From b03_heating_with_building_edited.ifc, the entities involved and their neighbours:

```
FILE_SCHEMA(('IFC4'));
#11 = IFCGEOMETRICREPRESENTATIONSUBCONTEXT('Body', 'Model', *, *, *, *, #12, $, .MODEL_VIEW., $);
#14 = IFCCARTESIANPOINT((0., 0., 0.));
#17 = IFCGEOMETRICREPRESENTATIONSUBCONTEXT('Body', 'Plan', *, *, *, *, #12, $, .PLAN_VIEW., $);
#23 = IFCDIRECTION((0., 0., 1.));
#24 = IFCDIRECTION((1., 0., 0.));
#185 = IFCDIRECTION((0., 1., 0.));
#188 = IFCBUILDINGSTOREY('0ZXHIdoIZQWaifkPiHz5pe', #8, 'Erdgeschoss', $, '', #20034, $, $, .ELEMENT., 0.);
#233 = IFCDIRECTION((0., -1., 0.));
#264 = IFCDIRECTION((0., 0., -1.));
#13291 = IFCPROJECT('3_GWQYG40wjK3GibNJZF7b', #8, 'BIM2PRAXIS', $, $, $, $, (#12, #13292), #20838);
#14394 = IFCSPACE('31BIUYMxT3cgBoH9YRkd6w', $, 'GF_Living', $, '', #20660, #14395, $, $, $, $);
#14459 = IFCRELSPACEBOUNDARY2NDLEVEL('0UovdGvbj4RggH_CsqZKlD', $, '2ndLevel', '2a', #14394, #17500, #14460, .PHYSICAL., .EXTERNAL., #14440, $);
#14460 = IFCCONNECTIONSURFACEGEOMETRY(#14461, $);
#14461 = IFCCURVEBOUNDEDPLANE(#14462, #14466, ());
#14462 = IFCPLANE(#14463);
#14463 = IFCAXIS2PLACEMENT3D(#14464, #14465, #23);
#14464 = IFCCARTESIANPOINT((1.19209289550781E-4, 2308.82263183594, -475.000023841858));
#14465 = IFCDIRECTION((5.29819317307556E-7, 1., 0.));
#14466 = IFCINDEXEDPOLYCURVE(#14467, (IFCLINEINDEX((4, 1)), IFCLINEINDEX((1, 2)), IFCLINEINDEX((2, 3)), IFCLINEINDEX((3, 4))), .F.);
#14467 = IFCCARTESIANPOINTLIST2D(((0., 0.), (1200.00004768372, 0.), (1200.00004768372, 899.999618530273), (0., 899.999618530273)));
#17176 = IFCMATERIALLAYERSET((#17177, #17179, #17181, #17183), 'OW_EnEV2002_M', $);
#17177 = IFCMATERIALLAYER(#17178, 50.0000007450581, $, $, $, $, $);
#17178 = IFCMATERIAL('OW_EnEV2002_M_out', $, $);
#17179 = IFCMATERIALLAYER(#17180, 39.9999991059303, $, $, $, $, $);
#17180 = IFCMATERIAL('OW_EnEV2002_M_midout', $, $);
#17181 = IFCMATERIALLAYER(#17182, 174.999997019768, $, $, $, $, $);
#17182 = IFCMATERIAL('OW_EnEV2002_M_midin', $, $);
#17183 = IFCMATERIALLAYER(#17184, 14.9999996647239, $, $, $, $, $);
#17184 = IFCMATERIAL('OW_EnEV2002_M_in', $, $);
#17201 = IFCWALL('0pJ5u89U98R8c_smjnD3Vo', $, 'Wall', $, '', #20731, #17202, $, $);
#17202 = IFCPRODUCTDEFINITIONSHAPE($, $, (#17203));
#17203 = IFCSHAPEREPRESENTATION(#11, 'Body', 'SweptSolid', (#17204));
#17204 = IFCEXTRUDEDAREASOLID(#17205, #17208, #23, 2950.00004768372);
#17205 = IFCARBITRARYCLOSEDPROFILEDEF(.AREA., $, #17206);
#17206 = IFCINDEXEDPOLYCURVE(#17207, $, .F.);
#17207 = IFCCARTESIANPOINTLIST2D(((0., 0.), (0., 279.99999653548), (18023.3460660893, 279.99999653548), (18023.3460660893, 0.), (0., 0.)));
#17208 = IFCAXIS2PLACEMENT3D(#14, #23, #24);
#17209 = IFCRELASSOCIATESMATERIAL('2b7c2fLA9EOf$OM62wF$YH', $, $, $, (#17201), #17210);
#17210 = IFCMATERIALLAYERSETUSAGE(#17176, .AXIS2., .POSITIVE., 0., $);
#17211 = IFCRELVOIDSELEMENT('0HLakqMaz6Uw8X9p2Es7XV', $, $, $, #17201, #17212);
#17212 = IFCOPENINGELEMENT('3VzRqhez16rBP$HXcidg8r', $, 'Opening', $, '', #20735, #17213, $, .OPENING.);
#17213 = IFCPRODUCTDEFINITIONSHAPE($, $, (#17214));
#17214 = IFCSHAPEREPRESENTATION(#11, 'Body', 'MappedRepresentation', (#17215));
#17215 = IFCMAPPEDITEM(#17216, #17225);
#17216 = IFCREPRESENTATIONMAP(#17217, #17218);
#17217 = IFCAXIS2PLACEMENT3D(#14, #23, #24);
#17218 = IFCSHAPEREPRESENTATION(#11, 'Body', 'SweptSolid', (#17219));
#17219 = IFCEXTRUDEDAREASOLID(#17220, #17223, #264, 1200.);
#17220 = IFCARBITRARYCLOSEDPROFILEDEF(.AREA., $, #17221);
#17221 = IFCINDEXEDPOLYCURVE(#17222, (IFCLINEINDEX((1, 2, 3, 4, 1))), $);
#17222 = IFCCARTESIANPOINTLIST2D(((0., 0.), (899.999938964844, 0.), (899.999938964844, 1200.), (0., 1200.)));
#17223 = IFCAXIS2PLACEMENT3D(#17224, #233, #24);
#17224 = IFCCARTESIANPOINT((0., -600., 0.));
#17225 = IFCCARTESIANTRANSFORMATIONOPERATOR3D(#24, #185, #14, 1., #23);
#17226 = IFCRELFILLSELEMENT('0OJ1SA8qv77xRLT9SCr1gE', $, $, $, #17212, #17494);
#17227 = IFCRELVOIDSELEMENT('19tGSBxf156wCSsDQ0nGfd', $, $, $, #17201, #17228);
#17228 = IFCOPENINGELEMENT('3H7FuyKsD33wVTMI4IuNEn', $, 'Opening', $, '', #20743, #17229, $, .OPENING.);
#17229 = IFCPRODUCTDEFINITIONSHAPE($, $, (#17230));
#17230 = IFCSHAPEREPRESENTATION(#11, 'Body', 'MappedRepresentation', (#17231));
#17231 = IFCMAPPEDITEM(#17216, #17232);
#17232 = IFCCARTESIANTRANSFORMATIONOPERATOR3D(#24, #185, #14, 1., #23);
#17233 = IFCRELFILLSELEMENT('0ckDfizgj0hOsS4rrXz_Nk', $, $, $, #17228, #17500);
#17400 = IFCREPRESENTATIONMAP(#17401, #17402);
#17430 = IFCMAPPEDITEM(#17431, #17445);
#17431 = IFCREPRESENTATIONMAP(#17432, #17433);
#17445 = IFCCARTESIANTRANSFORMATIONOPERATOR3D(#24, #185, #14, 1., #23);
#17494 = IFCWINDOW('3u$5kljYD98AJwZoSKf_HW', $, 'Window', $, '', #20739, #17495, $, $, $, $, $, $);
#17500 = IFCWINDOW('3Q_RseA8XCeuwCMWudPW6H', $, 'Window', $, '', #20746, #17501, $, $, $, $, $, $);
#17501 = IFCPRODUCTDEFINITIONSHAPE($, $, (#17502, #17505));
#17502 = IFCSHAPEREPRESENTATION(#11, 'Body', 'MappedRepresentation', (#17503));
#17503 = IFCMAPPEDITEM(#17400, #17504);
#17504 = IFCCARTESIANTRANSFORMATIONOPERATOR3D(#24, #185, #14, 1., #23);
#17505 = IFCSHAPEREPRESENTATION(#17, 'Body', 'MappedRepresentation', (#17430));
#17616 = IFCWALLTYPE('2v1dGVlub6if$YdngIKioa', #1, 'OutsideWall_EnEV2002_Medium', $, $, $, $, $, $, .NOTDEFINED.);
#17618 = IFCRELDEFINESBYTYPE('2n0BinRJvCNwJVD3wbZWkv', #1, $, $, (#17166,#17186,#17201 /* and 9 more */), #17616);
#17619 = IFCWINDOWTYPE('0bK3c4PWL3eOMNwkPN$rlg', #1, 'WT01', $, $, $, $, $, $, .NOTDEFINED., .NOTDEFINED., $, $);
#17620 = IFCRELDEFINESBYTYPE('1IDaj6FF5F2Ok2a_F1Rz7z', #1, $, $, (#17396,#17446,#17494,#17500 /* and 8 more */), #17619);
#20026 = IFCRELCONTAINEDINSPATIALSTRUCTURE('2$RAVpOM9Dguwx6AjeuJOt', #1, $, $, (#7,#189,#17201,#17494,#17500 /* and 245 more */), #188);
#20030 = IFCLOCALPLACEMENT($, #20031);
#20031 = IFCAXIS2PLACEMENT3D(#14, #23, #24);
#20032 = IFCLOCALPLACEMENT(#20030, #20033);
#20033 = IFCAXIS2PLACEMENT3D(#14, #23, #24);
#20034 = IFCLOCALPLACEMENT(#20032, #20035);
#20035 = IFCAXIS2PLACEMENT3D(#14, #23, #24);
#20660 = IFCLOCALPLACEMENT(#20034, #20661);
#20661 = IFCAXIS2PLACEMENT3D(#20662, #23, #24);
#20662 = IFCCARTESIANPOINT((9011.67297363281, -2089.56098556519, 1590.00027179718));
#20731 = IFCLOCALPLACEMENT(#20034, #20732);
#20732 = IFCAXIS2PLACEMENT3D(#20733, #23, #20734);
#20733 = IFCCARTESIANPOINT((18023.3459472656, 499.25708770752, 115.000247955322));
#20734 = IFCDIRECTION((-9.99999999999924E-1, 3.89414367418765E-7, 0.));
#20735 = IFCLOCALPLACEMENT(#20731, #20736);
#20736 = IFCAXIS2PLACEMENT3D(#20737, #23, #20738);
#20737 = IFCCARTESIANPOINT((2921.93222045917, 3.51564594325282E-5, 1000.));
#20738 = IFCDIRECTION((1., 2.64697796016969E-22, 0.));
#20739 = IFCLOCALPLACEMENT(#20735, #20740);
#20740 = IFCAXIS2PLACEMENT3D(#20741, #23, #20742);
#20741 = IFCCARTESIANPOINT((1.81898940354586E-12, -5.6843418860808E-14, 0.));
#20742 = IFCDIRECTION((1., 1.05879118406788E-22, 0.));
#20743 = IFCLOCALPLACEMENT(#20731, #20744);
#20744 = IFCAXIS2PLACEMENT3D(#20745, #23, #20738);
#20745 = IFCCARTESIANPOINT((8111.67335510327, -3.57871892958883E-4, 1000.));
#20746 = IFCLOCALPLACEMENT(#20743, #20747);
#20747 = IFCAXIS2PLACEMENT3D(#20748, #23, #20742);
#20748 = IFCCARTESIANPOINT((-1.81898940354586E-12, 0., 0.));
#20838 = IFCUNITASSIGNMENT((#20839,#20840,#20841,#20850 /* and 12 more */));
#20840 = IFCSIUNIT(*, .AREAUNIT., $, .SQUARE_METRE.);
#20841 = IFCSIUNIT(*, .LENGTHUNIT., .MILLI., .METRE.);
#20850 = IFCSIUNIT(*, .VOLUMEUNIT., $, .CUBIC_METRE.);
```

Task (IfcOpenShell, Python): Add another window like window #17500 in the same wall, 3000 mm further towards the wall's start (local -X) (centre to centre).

```python
import numpy as np
import ifcopenshell
import ifcopenshell.api.feature
import ifcopenshell.api.geometry
import ifcopenshell.api.root
import ifcopenshell.geom
import ifcopenshell.util.element
import ifcopenshell.util.placement
import ifcopenshell.util.shape

model = ifcopenshell.open("b03_heating_with_building_edited.ifc")
settings = ifcopenshell.geom.settings()


def volume(element):
    """Net volume in cubic metres, openings subtracted."""
    shape = ifcopenshell.geom.create_shape(settings, element)
    return ifcopenshell.util.shape.get_volume(shape.geometry)


def reuse_history(source, copy):
    """copy_class also copies each property set's owner history, people and application; keep the originals."""
    for rel in copy.IsDefinedBy:
        if rel.is_a("IfcRelDefinesByProperties") and (history := rel.RelatingPropertyDefinition.OwnerHistory):
            rel.RelatingPropertyDefinition.OwnerHistory = source.OwnerHistory
            ifcopenshell.util.element.remove_deep2(model, history)


window = model.by_guid("3Q_RseA8XCeuwCMWudPW6H")
opening = window.FillsVoids[0].RelatingOpeningElement
wall = opening.VoidsElements[0].RelatingBuildingElement
before = volume(wall)
shift = ifcopenshell.util.placement.get_local_placement(wall.ObjectPlacement)[:3, 0] * -3000.0

# copy_class copies the void relationship, type, container and properties, but no geometry.
new_opening = ifcopenshell.api.root.copy_class(model, product=opening)
new_opening.Representation = ifcopenshell.util.element.copy_deep(
    model, opening.Representation, exclude=["IfcGeometricRepresentationContext", "IfcRepresentationMap"]
)
reuse_history(opening, new_opening)
new_window = ifcopenshell.api.root.copy_class(model, product=window)
new_window.Representation = ifcopenshell.util.element.copy_deep(
    model, window.Representation, exclude=["IfcGeometricRepresentationContext", "IfcRepresentationMap"]
)
reuse_history(window, new_window)
ifcopenshell.api.feature.add_filling(model, opening=new_opening, element=new_window)

for old, new in ((opening, new_opening), (window, new_window)):
    matrix = ifcopenshell.util.placement.get_local_placement(old.ObjectPlacement)
    matrix[:3, 3] += shift
    ifcopenshell.api.geometry.edit_object_placement(model, product=new, matrix=matrix, is_si=False)

# The copied space boundaries still share their surfaces with the original.
for rel in new_window.ProvidesBoundaries:
    if rel.ConnectionGeometry:
        rel.ConnectionGeometry = ifcopenshell.util.element.copy_deep(model, rel.ConnectionGeometry)

# Space boundary surfaces are stored in each space's coordinates; move them too.
for rel in new_window.ProvidesBoundaries:
    if not rel.ConnectionGeometry:
        continue
    surface = rel.ConnectionGeometry.SurfaceOnRelatingElement.BasisSurface
    space_matrix = ifcopenshell.util.placement.get_local_placement(rel.RelatingSpace.ObjectPlacement)
    point = np.array(surface.Position.Location.Coordinates) + space_matrix[:3, :3].T @ shift
    surface.Position = model.createIfcAxis2Placement3D(
        model.createIfcCartesianPoint(point.tolist()), surface.Position.Axis, surface.Position.RefDirection
    )

after = volume(wall)

print(f"wall volume {before:.3f} -> {after:.3f} m3")

model.write("b03_heating_with_building_edited_edited.ifc")
```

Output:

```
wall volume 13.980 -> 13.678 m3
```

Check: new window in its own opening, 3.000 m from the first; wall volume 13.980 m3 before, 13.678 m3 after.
